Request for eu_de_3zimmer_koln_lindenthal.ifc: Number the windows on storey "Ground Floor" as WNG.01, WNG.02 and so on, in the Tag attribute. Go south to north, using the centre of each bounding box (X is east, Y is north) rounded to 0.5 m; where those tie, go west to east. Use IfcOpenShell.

First a look at what the model holds.

```python
import ifcopenshell
import ifcopenshell.util.element
import ifcopenshell.util.placement

model = ifcopenshell.open("eu_de_3zimmer_koln_lindenthal.ifc")
print(model.schema)
storey = next(s for s in model.by_type("IfcBuildingStorey") if s.Name == "Ground Floor")
windows = [e for e in ifcopenshell.util.element.get_decomposition(storey) if e.is_a("IfcWindow")]
for e in sorted(windows, key=lambda e: e.id()):
    origin = ifcopenshell.util.placement.get_local_placement(e.ObjectPlacement)[:3, 3]
    print(e.id(), e.Tag, e.Name, origin.round(2) + 0.0, sep=" | ")
```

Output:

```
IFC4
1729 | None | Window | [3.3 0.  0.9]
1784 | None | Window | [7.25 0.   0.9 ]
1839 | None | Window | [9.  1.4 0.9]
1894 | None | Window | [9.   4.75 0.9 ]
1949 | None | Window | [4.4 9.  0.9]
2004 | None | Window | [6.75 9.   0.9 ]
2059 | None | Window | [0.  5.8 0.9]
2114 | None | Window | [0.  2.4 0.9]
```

```python
import ifcopenshell
import ifcopenshell.geom
import ifcopenshell.util.element
import ifcopenshell.util.shape

model = ifcopenshell.open("eu_de_3zimmer_koln_lindenthal.ifc")
settings = ifcopenshell.geom.settings()
settings.set("use-world-coords", True)


def centre(element):
    shape = ifcopenshell.geom.create_shape(settings, element)
    return ifcopenshell.util.shape.get_bbox_centroid(shape.geometry)


storey = next(s for s in model.by_type("IfcBuildingStorey") if s.Name == "Ground Floor")
windows = [e for e in ifcopenshell.util.element.get_decomposition(storey) if e.is_a("IfcWindow")]

# Insertion points can sit at a corner or the storey origin, so sort by the geometry (in metres).
centres = {e: centre(e) for e in windows}
windows.sort(key=lambda e: (round(centres[e][1] / 0.5), centres[e][0]))

for i, e in enumerate(windows, start=1):
    number = f"WNG.{i:02d}"
    e.Tag = number
    print(e.id(), number)

model.write("eu_de_3zimmer_koln_lindenthal_rev.ifc")
```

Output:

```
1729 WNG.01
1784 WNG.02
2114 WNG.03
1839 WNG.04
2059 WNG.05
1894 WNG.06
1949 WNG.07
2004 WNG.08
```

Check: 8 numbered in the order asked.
